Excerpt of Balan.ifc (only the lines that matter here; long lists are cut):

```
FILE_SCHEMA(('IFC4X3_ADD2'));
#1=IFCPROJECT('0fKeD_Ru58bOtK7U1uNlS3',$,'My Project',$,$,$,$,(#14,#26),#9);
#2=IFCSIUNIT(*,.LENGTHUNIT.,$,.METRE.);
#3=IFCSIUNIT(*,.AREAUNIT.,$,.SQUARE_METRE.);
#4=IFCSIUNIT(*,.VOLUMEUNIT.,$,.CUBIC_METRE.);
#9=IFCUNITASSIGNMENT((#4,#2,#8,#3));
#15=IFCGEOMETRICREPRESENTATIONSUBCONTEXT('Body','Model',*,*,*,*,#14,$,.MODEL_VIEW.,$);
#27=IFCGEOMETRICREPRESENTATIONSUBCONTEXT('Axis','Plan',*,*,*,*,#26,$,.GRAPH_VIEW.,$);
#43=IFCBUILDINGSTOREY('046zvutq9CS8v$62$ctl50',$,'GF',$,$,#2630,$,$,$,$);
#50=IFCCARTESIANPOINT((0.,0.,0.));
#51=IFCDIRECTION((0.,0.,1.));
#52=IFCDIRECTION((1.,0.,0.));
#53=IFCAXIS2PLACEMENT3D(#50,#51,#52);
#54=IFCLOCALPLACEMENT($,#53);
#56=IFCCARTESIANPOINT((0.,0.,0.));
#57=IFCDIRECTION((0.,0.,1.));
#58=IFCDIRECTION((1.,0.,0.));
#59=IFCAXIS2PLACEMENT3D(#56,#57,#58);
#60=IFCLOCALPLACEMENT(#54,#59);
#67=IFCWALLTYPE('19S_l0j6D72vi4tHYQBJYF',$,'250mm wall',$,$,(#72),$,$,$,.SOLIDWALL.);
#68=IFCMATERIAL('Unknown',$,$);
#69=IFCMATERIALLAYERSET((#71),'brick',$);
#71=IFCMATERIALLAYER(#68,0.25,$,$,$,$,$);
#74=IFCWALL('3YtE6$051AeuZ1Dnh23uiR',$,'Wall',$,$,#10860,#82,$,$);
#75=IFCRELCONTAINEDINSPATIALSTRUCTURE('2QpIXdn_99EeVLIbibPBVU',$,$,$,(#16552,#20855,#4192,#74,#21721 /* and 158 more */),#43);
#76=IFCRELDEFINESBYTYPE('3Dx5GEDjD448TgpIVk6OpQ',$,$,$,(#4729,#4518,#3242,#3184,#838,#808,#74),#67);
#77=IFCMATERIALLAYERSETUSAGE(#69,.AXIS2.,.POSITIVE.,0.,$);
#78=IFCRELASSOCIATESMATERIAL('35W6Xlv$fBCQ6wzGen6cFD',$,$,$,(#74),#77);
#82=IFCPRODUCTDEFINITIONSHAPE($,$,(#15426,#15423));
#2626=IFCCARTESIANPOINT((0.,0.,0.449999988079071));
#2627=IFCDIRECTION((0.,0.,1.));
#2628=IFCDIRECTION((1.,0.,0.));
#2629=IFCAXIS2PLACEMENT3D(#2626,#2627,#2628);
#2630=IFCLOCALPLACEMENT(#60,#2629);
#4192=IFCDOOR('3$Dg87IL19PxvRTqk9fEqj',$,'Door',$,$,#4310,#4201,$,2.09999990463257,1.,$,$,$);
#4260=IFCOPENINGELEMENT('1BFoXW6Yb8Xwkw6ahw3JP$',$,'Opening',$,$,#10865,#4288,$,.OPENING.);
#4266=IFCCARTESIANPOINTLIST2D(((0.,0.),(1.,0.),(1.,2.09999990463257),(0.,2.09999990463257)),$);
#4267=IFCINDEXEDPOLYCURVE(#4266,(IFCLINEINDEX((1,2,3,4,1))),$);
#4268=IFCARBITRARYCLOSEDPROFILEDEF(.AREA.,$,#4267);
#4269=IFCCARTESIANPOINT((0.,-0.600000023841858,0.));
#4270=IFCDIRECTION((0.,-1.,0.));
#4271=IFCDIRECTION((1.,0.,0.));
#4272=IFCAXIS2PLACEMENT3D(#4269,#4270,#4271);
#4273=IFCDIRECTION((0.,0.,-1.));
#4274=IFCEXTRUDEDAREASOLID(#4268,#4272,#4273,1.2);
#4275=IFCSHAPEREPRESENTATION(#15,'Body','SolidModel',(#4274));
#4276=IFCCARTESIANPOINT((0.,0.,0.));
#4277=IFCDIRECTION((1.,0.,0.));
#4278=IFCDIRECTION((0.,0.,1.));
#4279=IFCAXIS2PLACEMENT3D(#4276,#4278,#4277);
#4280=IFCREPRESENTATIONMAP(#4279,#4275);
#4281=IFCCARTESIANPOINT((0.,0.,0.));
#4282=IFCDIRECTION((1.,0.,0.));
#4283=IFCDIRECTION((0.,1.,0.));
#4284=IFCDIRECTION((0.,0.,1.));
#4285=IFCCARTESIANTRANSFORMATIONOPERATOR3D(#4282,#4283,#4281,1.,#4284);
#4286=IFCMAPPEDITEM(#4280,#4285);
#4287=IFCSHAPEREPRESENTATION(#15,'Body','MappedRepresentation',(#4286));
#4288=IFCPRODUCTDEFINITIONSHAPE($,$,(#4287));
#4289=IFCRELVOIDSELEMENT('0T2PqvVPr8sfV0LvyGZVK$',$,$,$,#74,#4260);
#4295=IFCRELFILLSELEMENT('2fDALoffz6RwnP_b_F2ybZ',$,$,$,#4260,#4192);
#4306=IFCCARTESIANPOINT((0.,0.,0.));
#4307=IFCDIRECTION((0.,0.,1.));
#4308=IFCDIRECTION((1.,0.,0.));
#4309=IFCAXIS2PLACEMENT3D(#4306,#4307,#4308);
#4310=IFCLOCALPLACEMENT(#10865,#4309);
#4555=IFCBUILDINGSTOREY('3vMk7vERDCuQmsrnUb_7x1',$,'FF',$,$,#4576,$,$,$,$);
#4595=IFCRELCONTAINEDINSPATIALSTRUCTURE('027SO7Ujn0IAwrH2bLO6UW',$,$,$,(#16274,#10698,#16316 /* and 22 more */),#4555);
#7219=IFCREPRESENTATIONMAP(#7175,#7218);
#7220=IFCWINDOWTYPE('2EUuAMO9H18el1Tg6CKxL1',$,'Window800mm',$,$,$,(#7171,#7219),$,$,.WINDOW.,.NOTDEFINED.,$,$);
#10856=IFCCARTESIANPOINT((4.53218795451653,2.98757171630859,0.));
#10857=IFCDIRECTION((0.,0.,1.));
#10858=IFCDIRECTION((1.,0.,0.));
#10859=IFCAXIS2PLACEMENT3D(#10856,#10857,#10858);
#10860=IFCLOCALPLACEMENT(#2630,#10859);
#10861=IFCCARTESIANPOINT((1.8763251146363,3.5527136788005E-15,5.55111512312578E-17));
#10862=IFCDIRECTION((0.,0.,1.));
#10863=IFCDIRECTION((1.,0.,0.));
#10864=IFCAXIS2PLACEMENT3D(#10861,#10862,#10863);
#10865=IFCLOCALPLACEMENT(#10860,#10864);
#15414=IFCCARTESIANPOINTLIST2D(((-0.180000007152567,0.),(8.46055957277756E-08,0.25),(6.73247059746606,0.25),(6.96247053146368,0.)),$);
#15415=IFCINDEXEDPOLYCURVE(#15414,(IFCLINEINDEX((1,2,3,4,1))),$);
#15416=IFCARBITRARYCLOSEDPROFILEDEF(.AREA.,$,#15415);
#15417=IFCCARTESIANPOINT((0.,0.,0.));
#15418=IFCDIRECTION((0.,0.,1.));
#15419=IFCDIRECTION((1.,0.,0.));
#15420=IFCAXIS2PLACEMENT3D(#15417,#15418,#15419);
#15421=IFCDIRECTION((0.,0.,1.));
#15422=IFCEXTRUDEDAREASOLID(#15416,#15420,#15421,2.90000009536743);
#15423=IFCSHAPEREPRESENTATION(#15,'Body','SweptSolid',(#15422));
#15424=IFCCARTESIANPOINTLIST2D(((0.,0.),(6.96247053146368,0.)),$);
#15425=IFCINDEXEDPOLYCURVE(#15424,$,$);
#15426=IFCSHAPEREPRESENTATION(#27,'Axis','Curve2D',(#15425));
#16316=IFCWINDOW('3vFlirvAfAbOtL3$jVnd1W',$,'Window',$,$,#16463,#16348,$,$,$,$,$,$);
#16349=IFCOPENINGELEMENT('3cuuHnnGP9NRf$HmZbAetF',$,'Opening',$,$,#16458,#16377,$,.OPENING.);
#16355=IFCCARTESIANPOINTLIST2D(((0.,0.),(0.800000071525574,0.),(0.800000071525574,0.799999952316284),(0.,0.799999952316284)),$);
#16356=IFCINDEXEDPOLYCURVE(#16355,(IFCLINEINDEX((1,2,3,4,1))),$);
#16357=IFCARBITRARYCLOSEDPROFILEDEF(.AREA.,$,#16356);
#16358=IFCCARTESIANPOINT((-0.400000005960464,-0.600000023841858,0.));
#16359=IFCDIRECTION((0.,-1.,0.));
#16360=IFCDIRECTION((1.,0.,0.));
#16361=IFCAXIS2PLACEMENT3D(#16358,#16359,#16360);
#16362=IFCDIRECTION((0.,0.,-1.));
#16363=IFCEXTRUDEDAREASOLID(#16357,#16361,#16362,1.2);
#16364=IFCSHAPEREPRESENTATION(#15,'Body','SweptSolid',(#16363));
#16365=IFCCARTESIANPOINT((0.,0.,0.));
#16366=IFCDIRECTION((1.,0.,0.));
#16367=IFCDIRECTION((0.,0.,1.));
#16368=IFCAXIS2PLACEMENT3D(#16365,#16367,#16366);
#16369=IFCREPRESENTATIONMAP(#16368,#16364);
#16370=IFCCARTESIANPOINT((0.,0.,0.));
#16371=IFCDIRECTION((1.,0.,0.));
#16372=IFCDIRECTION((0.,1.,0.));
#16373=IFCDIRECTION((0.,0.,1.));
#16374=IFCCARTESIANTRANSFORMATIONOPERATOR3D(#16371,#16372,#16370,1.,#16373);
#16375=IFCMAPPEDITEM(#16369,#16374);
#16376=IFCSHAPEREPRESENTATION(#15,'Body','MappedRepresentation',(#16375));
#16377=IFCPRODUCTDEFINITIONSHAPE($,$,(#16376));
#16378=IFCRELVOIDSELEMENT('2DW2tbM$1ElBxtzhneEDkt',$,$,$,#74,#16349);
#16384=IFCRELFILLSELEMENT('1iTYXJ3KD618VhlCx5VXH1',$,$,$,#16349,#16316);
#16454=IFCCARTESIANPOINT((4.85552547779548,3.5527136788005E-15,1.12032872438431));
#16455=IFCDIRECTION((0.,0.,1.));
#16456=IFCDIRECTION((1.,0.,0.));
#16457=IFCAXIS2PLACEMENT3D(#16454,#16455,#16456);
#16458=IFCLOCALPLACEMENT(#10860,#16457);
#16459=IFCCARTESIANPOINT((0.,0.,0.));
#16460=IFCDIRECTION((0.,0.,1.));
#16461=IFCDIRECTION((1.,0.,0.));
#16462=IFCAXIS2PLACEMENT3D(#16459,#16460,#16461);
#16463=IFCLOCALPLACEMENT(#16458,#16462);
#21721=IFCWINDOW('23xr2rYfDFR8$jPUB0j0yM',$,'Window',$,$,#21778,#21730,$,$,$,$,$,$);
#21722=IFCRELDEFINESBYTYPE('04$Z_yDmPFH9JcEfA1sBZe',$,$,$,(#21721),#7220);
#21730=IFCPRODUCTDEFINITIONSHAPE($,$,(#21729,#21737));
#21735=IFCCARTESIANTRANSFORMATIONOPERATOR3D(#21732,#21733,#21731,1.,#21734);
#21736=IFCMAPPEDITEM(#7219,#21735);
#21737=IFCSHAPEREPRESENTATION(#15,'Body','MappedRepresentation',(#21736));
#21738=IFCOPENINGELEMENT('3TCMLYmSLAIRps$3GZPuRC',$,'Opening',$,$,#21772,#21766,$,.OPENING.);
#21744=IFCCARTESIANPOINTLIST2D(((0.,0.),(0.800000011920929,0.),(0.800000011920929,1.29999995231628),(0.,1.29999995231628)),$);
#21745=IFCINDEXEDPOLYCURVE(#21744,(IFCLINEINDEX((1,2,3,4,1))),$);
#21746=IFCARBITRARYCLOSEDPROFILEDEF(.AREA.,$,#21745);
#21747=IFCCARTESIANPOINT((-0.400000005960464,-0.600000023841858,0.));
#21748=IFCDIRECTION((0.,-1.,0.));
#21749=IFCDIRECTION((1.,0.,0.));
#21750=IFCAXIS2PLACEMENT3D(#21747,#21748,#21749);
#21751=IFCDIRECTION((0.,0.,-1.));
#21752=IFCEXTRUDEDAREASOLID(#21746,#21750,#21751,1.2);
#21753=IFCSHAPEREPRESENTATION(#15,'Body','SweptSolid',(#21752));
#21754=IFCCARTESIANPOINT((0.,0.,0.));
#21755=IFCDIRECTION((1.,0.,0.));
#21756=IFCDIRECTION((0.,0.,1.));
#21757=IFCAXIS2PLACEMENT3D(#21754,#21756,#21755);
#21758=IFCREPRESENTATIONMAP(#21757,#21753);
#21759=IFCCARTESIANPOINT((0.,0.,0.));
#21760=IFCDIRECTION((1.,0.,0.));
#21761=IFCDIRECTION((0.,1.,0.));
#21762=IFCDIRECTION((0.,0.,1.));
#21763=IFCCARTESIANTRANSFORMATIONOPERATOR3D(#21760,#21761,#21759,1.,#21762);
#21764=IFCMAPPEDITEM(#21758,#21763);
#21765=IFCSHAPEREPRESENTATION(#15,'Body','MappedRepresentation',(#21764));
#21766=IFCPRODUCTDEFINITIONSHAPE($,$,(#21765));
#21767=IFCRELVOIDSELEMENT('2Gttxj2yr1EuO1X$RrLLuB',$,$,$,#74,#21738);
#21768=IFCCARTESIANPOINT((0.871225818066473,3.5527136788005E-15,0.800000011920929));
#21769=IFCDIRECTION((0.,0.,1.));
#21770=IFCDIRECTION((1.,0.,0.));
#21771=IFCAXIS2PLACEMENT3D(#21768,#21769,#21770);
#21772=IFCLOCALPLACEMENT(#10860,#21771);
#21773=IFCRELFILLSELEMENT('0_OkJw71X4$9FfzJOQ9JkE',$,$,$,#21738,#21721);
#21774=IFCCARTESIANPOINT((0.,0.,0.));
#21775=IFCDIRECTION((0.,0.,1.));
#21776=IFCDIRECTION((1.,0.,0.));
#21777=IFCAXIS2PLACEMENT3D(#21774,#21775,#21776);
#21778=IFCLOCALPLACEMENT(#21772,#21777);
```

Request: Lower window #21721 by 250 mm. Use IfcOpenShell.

```python
import numpy as np
import ifcopenshell
import ifcopenshell.api.geometry
import ifcopenshell.util.placement
import ifcopenshell.util.unit

model = ifcopenshell.open("Balan.ifc")
unit_scale = ifcopenshell.util.unit.calculate_unit_scale(model)

window = model.by_guid("23xr2rYfDFR8$jPUB0j0yM")
opening = window.FillsVoids[0].RelatingOpeningElement
dz = -0.25 / unit_scale

shift = np.array([0.0, 0.0, dz])
# The window is placed relative to its opening, so it follows when the opening moves.
matrix = ifcopenshell.util.placement.get_local_placement(opening.ObjectPlacement)
matrix[:3, 3] += shift
ifcopenshell.api.geometry.edit_object_placement(
    model, product=opening, matrix=matrix, is_si=False, should_transform_children=True
)

print(f"moved by {dz * unit_scale:+.3f} m")

model.write("Balan-out.ifc")
```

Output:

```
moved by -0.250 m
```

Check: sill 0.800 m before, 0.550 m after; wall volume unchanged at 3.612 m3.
